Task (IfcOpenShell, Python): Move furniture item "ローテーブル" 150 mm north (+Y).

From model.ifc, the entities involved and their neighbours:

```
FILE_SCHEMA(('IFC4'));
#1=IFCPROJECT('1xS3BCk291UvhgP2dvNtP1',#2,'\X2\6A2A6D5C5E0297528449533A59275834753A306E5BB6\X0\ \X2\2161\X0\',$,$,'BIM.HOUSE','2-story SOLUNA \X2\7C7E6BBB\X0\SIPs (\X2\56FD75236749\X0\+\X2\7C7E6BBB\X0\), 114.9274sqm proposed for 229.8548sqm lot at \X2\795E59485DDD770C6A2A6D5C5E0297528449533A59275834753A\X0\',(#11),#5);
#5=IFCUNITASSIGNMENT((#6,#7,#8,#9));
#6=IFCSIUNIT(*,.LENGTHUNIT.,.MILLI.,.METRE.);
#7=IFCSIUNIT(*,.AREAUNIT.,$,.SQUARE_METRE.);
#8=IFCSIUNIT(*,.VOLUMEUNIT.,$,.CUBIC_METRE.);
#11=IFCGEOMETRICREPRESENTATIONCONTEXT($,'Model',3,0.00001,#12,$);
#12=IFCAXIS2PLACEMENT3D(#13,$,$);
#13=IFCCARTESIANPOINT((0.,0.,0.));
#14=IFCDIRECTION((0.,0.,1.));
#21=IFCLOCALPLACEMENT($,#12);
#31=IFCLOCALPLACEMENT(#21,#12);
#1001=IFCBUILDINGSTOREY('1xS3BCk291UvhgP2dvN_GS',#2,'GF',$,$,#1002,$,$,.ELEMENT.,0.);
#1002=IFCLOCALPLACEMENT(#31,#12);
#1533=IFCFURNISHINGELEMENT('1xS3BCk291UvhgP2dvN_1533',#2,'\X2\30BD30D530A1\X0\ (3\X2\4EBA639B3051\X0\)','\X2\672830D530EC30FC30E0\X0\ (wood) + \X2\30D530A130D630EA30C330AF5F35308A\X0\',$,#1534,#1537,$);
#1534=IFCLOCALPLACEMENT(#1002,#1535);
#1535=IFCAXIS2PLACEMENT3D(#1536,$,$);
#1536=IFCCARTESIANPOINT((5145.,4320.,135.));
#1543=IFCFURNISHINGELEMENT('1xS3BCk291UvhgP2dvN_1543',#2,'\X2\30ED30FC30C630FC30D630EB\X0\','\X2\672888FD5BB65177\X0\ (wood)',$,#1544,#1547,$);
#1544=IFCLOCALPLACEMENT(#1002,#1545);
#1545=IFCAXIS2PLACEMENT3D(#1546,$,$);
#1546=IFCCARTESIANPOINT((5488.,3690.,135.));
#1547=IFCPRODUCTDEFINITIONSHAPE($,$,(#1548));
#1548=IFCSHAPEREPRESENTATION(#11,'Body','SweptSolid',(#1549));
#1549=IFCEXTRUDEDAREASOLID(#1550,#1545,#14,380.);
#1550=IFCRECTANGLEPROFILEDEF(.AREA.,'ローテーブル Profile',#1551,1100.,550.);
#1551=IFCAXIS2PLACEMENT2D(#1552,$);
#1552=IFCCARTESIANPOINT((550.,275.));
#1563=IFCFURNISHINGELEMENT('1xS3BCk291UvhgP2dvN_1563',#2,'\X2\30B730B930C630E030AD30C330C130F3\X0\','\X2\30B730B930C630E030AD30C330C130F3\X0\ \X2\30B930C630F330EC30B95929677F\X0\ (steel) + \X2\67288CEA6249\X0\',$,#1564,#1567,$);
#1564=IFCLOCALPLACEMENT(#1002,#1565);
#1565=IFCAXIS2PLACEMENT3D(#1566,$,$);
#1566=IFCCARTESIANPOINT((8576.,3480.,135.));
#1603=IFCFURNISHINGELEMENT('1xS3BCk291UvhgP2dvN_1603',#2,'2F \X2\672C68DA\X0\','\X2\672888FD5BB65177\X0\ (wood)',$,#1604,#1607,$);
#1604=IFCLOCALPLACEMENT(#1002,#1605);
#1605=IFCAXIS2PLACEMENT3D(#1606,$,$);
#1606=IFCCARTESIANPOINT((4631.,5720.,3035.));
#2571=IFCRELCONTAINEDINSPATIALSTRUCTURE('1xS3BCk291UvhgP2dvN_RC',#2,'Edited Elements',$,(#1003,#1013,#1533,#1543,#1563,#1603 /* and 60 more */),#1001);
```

```python
import ifcopenshell
import ifcopenshell.api.geometry
import ifcopenshell.util.placement

model = ifcopenshell.open("model.ifc")

item = model.by_guid("1xS3BCk291UvhgP2dvN_1543")
matrix = ifcopenshell.util.placement.get_local_placement(item.ObjectPlacement)
matrix[1, 3] += 150.0
ifcopenshell.api.geometry.edit_object_placement(model, product=item, matrix=matrix, is_si=False)

print(ifcopenshell.util.placement.get_local_placement(item.ObjectPlacement).round(3) + 0.0)

model.write("model_v2.ifc")
```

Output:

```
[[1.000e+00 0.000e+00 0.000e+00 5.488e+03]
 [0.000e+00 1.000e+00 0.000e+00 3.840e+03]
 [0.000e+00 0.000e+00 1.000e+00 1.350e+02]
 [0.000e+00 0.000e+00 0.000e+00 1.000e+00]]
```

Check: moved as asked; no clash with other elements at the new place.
